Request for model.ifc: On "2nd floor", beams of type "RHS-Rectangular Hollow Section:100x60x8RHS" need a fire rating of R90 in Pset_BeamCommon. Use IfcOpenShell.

First a look at what the model holds.

```python
import ifcopenshell
import ifcopenshell.util.element

model = ifcopenshell.open("model.ifc")
print(model.schema)
storey = next(s for s in model.by_type("IfcBuildingStorey") if s.Name == "2nd floor")
beams = [e for e in ifcopenshell.util.element.get_decomposition(storey) if e.is_a("IfcBeam")]
seen = {}
for e in beams:
    element_type = ifcopenshell.util.element.get_type(e)
    key = (element_type.Name if element_type != e and element_type else None, ifcopenshell.util.element.get_pset(e, "Pset_BeamCommon", "FireRating"))
    seen[key] = seen.get(key, 0) + 1
for (name, value), count in sorted(seen.items(), key=str):
    print(count, "x", name, "|", value)
```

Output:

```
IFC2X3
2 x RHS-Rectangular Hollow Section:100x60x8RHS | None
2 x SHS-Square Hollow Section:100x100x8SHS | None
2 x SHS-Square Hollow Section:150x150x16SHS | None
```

```python
import ifcopenshell
import ifcopenshell.api.pset
import ifcopenshell.util.element

model = ifcopenshell.open("model.ifc")

storey = next(s for s in model.by_type("IfcBuildingStorey") if s.Name == "2nd floor")
beams = [e for e in ifcopenshell.util.element.get_decomposition(storey) if e.is_a("IfcBeam")]

count = 0
for e in beams:
    element_type = ifcopenshell.util.element.get_type(e)
    if element_type in (None, e) or element_type.Name != "RHS-Rectangular Hollow Section:100x60x8RHS":
        continue
    # add_pset returns the element's existing set when there is one.
    pset = ifcopenshell.api.pset.add_pset(model, product=e, name="Pset_BeamCommon")
    ifcopenshell.api.pset.edit_pset(model, pset=pset, properties={"FireRating": "R90"})
    count += 1

print(count, "beams updated")

model.write("model_edited.ifc")
```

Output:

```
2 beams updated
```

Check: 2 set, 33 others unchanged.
